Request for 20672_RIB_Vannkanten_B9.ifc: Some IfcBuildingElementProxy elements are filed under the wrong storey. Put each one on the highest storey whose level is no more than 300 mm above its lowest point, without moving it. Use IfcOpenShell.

First a look at what the model holds.

```python
import ifcopenshell
import ifcopenshell.util.element
import ifcopenshell.util.placement

model = ifcopenshell.open("20672_RIB_Vannkanten_B9.ifc")
print(model.schema)
for storey in model.by_type("IfcBuildingStorey"):
    level = ifcopenshell.util.placement.get_storey_elevation(storey)
    count = sum(e.is_a("IfcBuildingElementProxy") for e in ifcopenshell.util.element.get_contained(storey))
    print(storey.id(), storey.Name, round(level, 3), count, sep=" | ")
```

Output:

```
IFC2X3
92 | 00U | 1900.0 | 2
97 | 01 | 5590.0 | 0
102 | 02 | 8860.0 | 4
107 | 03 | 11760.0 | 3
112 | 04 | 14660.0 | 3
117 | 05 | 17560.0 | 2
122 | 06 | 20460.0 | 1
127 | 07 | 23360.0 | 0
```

```python
import ifcopenshell
import ifcopenshell.api.spatial
import ifcopenshell.geom
import ifcopenshell.util.element
import ifcopenshell.util.placement
import ifcopenshell.util.shape
import ifcopenshell.util.unit

model = ifcopenshell.open("20672_RIB_Vannkanten_B9.ifc")
unit_scale = ifcopenshell.util.unit.calculate_unit_scale(model)
settings = ifcopenshell.geom.settings()

levels = sorted(
    ((ifcopenshell.util.placement.get_storey_elevation(s) * unit_scale, s) for s in model.by_type("IfcBuildingStorey")),
    key=lambda pair: pair[0],
)

for e in model.by_type("IfcBuildingElementProxy"):
    current = e.ContainedInStructure[0].RelatingStructure if e.ContainedInStructure else None
    if current is None or not current.is_a("IfcBuildingStorey"):
        continue
    shape = ifcopenshell.geom.create_shape(settings, e)
    bottom = ifcopenshell.util.shape.get_shape_bottom_elevation(shape, shape.geometry)
    below = [s for level, s in levels if level <= bottom + 0.3]
    storey = below[-1] if below else levels[0][1]
    if storey != current:
        # assign_container keeps the world position.
        ifcopenshell.api.spatial.assign_container(model, products=[e], relating_structure=storey)
        print(e.id(), current.Name, "->", storey.Name)

model.write("20672_RIB_Vannkanten_B9_edited.ifc")
```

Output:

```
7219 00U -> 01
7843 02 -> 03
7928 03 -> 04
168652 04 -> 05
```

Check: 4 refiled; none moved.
